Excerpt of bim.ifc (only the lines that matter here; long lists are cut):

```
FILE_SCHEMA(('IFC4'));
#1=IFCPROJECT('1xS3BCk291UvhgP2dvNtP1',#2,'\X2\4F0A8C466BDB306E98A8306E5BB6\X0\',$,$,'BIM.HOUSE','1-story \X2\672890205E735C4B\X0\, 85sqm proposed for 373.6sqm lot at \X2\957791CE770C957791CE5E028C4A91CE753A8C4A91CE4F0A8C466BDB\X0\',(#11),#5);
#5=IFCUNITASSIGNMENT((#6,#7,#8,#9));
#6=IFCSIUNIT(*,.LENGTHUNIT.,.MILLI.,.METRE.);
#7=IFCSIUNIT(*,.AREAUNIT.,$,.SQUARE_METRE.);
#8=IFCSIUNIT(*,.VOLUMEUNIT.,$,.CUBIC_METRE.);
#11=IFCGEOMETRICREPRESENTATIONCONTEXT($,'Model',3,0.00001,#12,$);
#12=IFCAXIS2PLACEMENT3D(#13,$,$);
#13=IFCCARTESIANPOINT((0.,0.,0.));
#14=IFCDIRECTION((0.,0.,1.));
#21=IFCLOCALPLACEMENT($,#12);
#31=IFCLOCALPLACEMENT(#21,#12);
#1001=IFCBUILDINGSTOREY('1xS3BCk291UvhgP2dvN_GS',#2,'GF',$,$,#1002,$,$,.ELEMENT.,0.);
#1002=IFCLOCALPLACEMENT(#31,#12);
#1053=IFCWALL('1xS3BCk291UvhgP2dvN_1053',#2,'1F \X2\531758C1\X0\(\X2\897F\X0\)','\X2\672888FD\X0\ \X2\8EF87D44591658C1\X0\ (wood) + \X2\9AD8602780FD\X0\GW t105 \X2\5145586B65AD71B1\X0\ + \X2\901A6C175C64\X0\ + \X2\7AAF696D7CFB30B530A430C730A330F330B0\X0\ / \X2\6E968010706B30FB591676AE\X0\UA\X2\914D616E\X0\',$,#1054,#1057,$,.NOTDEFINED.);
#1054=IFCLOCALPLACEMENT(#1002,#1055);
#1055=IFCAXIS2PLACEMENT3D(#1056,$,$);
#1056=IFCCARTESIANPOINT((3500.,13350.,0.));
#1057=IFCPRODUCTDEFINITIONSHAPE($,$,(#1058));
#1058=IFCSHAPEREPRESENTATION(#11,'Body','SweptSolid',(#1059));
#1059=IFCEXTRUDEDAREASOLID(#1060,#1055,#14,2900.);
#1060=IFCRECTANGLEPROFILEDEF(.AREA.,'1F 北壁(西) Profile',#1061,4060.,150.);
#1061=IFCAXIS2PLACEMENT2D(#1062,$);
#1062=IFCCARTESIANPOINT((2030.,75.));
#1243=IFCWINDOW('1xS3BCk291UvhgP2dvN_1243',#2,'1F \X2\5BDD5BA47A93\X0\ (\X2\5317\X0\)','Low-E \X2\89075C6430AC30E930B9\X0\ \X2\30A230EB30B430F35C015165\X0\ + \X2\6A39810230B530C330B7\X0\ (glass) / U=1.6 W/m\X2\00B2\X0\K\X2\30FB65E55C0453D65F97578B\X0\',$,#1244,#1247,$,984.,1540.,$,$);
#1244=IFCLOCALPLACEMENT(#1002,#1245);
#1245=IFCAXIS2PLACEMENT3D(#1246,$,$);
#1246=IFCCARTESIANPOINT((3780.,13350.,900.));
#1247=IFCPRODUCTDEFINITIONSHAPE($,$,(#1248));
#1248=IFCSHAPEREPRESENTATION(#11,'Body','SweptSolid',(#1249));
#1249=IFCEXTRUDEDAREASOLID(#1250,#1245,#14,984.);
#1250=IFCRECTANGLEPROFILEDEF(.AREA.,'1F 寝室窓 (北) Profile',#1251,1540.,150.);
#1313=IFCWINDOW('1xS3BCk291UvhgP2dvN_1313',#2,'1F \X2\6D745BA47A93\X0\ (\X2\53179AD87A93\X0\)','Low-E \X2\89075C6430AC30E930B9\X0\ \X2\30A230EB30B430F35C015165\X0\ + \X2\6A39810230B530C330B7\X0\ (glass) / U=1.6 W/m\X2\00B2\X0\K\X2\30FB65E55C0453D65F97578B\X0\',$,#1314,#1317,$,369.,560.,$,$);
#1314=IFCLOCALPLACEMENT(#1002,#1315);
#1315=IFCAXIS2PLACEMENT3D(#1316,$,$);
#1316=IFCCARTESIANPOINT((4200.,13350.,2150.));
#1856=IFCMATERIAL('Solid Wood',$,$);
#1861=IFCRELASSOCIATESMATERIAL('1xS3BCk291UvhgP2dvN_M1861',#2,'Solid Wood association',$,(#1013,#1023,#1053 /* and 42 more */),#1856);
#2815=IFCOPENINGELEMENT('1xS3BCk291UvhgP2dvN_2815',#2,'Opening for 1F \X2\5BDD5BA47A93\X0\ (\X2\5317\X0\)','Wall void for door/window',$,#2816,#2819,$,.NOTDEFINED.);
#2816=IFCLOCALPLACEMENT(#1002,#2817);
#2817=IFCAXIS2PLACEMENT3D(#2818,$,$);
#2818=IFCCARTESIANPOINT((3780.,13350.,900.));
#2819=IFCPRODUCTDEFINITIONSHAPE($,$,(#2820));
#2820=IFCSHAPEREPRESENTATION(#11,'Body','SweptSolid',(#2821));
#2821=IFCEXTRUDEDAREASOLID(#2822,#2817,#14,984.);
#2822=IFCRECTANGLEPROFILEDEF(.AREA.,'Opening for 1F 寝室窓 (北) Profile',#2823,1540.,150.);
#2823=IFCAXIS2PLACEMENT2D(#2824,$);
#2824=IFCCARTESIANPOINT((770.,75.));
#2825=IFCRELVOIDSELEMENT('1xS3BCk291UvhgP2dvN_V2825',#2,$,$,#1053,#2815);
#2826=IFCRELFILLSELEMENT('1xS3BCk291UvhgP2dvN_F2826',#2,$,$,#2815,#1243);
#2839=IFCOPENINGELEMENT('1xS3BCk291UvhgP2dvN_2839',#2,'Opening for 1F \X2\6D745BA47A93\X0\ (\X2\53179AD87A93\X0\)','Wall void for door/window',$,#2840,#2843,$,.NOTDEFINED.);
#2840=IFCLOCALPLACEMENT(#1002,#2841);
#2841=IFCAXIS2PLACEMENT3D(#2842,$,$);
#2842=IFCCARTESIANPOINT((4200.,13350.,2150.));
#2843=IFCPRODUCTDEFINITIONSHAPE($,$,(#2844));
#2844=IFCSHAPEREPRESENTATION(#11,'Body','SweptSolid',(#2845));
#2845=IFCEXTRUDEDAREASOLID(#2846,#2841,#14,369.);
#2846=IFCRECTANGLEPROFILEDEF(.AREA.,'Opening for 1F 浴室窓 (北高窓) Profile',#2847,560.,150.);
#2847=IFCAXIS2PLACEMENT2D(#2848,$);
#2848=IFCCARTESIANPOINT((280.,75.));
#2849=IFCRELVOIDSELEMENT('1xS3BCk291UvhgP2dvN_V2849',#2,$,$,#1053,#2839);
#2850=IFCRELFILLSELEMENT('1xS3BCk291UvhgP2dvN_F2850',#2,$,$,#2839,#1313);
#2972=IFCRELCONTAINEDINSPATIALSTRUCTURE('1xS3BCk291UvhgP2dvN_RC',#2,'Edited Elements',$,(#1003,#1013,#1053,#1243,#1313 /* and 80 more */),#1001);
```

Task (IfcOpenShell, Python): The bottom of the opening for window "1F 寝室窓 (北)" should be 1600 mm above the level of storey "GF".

```python
import numpy as np
import ifcopenshell
import ifcopenshell.api.geometry
import ifcopenshell.geom
import ifcopenshell.util.element
import ifcopenshell.util.placement
import ifcopenshell.util.shape
import ifcopenshell.util.unit

model = ifcopenshell.open("bim.ifc")
unit_scale = ifcopenshell.util.unit.calculate_unit_scale(model)

window = model.by_guid("1xS3BCk291UvhgP2dvN_1243")
opening = window.FillsVoids[0].RelatingOpeningElement
storey = ifcopenshell.util.element.get_container(window, ifc_class="IfcBuildingStorey")
level = ifcopenshell.util.placement.get_local_placement(storey.ObjectPlacement)[2, 3]

# The opening's origin need not be at the sill, so measure its lowest point.
shape = ifcopenshell.geom.create_shape(ifcopenshell.geom.settings(), opening)
bottom = ifcopenshell.util.shape.get_shape_bottom_elevation(shape, shape.geometry) / unit_scale
dz = level + 1600.0 - bottom

shift = np.array([0.0, 0.0, dz])
# The window is not placed relative to its opening, so move both.
for product in (opening, window):
    matrix = ifcopenshell.util.placement.get_local_placement(product.ObjectPlacement)
    matrix[:3, 3] += shift
    ifcopenshell.api.geometry.edit_object_placement(model, product=product, matrix=matrix, is_si=False)

print(f"moved by {dz * unit_scale:+.3f} m")

model.write("bim_rev.ifc")
```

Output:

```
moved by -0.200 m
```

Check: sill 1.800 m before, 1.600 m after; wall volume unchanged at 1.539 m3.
